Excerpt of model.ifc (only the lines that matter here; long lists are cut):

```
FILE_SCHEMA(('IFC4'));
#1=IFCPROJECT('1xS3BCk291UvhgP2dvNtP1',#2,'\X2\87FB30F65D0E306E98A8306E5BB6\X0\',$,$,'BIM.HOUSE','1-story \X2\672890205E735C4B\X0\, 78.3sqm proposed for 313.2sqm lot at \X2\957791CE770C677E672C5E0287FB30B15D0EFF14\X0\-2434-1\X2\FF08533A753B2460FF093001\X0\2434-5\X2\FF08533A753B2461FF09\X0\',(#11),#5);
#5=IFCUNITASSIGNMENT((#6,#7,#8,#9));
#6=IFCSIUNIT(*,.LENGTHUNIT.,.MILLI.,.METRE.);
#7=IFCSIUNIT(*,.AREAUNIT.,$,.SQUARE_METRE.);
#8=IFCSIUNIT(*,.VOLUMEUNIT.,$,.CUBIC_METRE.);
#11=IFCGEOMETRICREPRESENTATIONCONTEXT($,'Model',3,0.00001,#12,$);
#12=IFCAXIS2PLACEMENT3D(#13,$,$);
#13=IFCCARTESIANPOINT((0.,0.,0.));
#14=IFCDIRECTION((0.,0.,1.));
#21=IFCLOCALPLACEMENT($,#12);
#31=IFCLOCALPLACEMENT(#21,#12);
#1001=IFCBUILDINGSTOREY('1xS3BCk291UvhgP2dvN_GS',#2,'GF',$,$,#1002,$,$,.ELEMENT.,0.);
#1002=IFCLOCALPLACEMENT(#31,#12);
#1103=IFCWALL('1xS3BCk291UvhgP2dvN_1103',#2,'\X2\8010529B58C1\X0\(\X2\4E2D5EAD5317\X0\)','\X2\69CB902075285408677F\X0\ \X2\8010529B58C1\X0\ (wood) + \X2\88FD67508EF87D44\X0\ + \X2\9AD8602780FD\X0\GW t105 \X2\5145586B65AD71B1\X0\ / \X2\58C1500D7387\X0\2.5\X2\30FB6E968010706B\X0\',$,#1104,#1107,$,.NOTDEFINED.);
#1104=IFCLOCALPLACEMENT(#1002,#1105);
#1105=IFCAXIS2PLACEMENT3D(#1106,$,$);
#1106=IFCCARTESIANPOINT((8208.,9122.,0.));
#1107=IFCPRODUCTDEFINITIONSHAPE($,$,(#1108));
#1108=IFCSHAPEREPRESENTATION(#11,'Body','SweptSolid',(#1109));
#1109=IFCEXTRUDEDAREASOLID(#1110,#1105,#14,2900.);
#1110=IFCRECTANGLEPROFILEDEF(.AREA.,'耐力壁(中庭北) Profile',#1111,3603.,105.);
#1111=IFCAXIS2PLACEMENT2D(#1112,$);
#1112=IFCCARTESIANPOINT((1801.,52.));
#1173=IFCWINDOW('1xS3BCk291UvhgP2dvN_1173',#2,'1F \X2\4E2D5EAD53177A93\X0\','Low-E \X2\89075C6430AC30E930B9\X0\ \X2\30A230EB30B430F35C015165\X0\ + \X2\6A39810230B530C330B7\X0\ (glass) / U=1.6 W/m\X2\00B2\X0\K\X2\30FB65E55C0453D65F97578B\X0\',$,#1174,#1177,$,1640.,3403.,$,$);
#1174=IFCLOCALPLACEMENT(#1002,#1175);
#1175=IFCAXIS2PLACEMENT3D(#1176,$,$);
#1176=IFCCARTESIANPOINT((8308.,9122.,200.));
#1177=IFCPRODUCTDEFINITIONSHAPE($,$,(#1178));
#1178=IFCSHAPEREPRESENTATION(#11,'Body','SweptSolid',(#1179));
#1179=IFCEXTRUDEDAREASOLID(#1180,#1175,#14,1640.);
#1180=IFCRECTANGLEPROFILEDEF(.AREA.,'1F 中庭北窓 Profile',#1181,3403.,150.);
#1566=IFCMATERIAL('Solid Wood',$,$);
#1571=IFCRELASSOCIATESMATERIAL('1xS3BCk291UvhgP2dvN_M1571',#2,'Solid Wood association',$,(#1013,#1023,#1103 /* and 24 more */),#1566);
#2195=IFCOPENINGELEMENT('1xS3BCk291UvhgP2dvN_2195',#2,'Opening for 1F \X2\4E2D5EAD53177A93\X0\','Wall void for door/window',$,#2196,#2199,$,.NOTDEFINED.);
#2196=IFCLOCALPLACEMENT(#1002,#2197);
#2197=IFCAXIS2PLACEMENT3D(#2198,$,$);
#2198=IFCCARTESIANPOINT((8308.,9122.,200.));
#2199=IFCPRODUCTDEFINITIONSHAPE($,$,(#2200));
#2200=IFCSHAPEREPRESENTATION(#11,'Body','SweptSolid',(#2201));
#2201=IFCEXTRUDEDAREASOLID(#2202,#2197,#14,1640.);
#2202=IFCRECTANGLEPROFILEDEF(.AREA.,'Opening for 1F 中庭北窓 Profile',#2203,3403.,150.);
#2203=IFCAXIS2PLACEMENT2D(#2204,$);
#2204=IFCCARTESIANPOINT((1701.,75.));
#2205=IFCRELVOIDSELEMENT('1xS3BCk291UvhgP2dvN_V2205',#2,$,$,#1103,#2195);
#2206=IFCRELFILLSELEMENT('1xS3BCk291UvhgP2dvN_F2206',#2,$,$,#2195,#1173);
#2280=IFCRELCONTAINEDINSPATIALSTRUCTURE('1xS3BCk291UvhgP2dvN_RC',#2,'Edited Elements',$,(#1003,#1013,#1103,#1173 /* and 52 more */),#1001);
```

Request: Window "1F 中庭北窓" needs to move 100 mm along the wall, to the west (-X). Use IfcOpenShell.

```python
import ifcopenshell
import ifcopenshell.api.geometry
import ifcopenshell.util.placement
import ifcopenshell.util.unit

model = ifcopenshell.open("model.ifc")
unit_scale = ifcopenshell.util.unit.calculate_unit_scale(model)

window = model.by_guid("1xS3BCk291UvhgP2dvN_1173")
opening = window.FillsVoids[0].RelatingOpeningElement
wall = opening.VoidsElements[0].RelatingBuildingElement

wall_matrix = ifcopenshell.util.placement.get_local_placement(wall.ObjectPlacement)
shift = wall_matrix[:3, 0] * -0.1 / unit_scale
before = ifcopenshell.util.placement.get_local_placement(window.ObjectPlacement)[:3, 3].copy()

# The window is not placed relative to its opening, so move both.
for product in (opening, window):
    matrix = ifcopenshell.util.placement.get_local_placement(product.ObjectPlacement)
    matrix[:3, 3] += shift
    ifcopenshell.api.geometry.edit_object_placement(model, product=product, matrix=matrix, is_si=False)

after = ifcopenshell.util.placement.get_local_placement(window.ObjectPlacement)[:3, 3]
print("window moved by", (after - before).round(3) + 0.0)

model.write("model_updated.ifc")
```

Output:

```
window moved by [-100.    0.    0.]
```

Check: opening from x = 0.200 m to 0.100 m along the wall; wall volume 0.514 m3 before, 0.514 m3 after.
